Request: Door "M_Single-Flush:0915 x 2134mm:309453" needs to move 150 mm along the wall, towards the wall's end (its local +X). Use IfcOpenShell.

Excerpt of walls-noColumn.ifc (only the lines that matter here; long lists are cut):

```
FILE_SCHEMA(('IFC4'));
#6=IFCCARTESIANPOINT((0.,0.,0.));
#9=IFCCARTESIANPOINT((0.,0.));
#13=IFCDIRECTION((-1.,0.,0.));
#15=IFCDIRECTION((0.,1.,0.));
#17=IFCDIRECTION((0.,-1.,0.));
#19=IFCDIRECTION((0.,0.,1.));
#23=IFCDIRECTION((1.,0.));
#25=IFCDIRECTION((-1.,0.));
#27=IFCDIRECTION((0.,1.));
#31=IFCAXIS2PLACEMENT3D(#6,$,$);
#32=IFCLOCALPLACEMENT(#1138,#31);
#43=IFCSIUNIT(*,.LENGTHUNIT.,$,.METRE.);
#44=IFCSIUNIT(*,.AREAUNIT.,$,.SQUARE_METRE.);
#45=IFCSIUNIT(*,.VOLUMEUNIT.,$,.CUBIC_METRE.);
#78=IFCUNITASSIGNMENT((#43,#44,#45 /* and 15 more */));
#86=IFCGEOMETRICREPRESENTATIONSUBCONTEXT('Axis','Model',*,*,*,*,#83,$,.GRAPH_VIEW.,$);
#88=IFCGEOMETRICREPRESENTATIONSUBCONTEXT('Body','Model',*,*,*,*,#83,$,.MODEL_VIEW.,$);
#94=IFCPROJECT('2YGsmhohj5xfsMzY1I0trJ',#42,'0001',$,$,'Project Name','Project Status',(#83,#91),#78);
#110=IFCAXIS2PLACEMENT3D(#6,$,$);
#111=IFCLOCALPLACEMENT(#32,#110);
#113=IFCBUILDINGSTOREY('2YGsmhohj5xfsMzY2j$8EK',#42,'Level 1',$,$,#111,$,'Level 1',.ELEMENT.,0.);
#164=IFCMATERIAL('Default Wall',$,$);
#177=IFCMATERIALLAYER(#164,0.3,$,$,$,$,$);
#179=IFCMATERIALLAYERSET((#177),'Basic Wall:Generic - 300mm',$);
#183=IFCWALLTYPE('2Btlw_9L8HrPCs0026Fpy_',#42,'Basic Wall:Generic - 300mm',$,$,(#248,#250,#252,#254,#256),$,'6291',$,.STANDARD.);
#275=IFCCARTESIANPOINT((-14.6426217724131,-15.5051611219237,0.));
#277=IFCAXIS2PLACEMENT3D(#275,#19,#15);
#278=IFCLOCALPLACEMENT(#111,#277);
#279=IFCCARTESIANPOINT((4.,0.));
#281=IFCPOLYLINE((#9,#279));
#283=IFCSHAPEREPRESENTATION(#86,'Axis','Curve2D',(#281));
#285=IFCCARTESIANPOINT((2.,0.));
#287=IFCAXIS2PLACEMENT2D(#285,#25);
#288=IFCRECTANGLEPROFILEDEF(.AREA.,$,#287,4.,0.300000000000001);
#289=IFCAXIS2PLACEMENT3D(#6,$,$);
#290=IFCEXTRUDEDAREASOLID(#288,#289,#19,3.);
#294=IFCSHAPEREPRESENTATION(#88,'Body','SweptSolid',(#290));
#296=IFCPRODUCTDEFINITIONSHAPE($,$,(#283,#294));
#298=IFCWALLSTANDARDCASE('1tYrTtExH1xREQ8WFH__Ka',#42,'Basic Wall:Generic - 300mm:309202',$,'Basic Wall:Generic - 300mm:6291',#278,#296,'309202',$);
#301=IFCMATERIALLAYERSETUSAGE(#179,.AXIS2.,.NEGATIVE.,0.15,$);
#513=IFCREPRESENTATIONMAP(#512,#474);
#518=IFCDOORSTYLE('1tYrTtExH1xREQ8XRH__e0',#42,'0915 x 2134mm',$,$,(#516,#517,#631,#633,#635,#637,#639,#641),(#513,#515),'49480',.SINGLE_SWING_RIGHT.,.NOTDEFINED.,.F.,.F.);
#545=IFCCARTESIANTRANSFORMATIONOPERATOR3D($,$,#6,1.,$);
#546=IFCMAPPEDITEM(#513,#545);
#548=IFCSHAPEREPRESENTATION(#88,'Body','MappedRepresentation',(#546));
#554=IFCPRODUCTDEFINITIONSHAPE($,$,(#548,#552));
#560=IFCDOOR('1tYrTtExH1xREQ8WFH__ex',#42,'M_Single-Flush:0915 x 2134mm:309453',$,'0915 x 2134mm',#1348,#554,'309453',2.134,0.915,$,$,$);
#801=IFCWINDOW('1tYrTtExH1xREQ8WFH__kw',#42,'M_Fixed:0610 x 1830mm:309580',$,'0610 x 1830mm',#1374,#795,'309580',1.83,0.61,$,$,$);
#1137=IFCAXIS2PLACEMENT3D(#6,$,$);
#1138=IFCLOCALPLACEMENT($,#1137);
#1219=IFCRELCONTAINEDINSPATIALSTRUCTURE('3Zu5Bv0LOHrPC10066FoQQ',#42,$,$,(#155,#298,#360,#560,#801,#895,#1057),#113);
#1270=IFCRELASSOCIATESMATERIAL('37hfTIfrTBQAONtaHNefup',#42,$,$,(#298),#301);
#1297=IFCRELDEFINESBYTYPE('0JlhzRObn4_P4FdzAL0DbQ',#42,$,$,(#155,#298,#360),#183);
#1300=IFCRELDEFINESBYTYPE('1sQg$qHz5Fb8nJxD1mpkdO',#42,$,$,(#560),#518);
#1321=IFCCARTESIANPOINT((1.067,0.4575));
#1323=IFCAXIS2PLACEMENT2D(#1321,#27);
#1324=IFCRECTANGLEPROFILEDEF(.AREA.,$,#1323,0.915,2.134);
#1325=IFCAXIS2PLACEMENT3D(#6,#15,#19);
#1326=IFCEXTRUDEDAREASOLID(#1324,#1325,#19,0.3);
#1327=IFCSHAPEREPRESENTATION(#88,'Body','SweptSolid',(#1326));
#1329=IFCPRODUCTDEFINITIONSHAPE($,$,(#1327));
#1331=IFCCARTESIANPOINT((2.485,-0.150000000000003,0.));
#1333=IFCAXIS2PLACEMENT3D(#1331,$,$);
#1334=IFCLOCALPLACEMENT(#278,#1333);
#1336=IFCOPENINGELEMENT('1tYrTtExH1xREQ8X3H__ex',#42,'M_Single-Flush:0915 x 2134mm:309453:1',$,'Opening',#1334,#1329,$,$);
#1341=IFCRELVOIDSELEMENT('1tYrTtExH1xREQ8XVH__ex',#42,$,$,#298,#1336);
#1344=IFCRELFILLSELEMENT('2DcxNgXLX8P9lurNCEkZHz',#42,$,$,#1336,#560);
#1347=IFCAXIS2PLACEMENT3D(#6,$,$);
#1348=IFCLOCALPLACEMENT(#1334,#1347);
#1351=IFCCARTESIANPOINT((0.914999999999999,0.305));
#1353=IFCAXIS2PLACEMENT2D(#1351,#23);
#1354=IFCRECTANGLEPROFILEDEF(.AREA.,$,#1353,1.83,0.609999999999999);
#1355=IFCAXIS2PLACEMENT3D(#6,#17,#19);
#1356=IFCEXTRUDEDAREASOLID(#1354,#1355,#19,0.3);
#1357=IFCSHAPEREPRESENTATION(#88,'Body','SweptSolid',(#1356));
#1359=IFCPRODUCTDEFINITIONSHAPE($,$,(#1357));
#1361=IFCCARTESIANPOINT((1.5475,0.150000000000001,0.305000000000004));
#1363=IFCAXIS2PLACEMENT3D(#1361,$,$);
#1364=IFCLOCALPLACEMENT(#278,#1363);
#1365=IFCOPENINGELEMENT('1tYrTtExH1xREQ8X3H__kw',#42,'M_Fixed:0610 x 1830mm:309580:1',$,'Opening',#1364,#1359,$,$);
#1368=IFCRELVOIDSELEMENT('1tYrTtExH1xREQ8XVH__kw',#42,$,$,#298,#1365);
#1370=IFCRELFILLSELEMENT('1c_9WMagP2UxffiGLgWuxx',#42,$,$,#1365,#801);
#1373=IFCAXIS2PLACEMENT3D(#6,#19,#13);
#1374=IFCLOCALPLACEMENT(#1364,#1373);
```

```python
import ifcopenshell
import ifcopenshell.api.geometry
import ifcopenshell.util.placement
import ifcopenshell.util.unit

model = ifcopenshell.open("walls-noColumn.ifc")
unit_scale = ifcopenshell.util.unit.calculate_unit_scale(model)

door = model.by_guid("1tYrTtExH1xREQ8WFH__ex")
opening = door.FillsVoids[0].RelatingOpeningElement
wall = opening.VoidsElements[0].RelatingBuildingElement

wall_matrix = ifcopenshell.util.placement.get_local_placement(wall.ObjectPlacement)
shift = wall_matrix[:3, 0] * 0.15 / unit_scale
before = ifcopenshell.util.placement.get_local_placement(door.ObjectPlacement)[:3, 3].copy()

# The door is placed relative to its opening, so it follows when the opening moves.
matrix = ifcopenshell.util.placement.get_local_placement(opening.ObjectPlacement)
matrix[:3, 3] += shift
ifcopenshell.api.geometry.edit_object_placement(
    model, product=opening, matrix=matrix, is_si=False, should_transform_children=True
)

after = ifcopenshell.util.placement.get_local_placement(door.ObjectPlacement)[:3, 3]
print("door moved by", (after - before).round(3) + 0.0)

model.write("walls-noColumn_rev.ifc")
```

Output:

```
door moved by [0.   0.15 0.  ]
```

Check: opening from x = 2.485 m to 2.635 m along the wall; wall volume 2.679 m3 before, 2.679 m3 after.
